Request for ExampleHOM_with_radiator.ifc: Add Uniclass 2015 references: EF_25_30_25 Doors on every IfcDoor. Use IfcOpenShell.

First a look at what the model holds.

```python
import ifcopenshell

model = ifcopenshell.open("ExampleHOM_with_radiator.ifc")
print(model.schema)
print("classifications:", [c.Name for c in model.by_type("IfcClassification")])
for ifc_class in ("IfcDoor", "IfcRoof", "IfcStair", "IfcWall", "IfcWindow"):
    print(ifc_class, len(model.by_type(ifc_class)))
```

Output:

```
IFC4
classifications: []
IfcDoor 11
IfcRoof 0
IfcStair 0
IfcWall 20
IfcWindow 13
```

```python
import ifcopenshell
import ifcopenshell.api.classification

model = ifcopenshell.open("ExampleHOM_with_radiator.ifc")

system = ifcopenshell.api.classification.add_classification(model, classification="Uniclass 2015")

codes = {
    "IfcDoor": ("EF_25_30_25", "Doors"),
}
for ifc_class, (code, name) in codes.items():
    products = model.by_type(ifc_class)
    ifcopenshell.api.classification.add_reference(
        model, products=products, classification=system, identification=code, name=name
    )
    print(code, len(products))

model.write("ExampleHOM_with_radiator_updated.ifc")
```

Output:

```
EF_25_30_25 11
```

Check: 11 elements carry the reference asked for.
